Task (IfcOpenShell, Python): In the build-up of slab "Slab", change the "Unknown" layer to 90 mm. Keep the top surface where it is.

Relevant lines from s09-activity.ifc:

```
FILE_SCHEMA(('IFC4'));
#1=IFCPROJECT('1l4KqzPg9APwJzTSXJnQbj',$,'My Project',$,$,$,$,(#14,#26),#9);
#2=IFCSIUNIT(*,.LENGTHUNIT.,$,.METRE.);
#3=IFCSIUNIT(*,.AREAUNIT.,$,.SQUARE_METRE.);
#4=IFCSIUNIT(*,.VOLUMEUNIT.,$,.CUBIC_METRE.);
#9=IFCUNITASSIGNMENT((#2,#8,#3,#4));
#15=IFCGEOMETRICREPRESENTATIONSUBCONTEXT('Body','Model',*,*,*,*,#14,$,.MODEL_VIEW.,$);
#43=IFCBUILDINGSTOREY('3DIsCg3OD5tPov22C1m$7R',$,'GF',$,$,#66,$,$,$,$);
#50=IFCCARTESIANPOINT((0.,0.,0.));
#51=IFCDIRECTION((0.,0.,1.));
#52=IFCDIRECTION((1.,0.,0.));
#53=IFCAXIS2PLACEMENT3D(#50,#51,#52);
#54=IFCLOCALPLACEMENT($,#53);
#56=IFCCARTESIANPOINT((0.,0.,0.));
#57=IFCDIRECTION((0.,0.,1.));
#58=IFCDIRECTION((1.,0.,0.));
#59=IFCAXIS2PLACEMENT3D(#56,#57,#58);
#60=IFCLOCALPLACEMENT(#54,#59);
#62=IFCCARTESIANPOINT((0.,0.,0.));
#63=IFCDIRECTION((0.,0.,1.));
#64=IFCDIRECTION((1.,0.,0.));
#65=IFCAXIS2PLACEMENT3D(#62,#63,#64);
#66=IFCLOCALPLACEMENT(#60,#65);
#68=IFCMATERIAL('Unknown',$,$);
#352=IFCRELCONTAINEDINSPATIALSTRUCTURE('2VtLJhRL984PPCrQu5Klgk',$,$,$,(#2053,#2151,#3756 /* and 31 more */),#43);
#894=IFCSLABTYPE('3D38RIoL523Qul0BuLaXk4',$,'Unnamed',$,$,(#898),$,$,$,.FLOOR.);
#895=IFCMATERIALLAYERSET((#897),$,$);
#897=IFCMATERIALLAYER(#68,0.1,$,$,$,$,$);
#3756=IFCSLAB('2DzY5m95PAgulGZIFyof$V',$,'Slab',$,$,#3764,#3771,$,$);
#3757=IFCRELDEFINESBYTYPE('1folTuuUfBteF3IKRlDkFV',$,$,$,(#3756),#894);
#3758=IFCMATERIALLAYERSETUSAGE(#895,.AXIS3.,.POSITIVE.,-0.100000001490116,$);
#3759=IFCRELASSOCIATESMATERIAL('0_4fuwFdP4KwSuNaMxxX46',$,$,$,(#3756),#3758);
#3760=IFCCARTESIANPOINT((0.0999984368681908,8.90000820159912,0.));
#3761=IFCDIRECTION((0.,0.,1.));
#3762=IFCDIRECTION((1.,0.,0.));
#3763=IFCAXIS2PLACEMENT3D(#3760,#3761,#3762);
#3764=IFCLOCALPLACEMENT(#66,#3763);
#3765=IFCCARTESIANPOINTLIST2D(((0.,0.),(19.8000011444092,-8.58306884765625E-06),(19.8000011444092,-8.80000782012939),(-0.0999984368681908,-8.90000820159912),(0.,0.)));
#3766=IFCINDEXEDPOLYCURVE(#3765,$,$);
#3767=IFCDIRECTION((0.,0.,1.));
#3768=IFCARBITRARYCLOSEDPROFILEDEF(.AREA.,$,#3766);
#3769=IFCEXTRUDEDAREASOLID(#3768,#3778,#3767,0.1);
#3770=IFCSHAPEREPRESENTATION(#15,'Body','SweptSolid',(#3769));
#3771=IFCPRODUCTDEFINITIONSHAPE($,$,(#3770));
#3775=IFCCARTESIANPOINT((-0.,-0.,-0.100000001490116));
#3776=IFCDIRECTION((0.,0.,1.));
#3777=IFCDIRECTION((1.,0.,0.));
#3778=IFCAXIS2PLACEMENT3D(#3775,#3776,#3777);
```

```python
import ifcopenshell
import ifcopenshell.util.element
import ifcopenshell.util.representation
import ifcopenshell.util.unit

model = ifcopenshell.open("s09-activity.ifc")
unit_scale = ifcopenshell.util.unit.calculate_unit_scale(model)

layer_set = model.by_id(895)
layer = next(l for l in layer_set.MaterialLayers if l.Material and l.Material.Name == "Unknown")
change = 0.09 / unit_scale - layer.LayerThickness
layer.LayerThickness += change

# Geometry does not follow the layer set by itself.
slabs = [e for e in ifcopenshell.util.element.get_elements_by_material(model, layer_set) if e.is_a("IfcSlab")]
for slab in sorted(slabs, key=lambda e: e.id()):
    body = ifcopenshell.util.representation.get_representation(slab, "Model", "Body")
    solid = body.Items[0]
    old_depth = solid.Depth
    solid.Depth += change
    # Extruded upwards: lower the start of the extrusion so the top stays.
    x, y, z = solid.Position.Location.Coordinates
    solid.Position.Location = model.createIfcCartesianPoint((x, y, z - change))
    print(slab.id(), f"{old_depth:g} -> {solid.Depth:g}")

# The layers are counted up from the underside, which has moved.
for usage in {ifcopenshell.util.element.get_material(slab) for slab in slabs}:
    usage.OffsetFromReferenceLine -= change

model.write("s09-activity-out.ifc")
```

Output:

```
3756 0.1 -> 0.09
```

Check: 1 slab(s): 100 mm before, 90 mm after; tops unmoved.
